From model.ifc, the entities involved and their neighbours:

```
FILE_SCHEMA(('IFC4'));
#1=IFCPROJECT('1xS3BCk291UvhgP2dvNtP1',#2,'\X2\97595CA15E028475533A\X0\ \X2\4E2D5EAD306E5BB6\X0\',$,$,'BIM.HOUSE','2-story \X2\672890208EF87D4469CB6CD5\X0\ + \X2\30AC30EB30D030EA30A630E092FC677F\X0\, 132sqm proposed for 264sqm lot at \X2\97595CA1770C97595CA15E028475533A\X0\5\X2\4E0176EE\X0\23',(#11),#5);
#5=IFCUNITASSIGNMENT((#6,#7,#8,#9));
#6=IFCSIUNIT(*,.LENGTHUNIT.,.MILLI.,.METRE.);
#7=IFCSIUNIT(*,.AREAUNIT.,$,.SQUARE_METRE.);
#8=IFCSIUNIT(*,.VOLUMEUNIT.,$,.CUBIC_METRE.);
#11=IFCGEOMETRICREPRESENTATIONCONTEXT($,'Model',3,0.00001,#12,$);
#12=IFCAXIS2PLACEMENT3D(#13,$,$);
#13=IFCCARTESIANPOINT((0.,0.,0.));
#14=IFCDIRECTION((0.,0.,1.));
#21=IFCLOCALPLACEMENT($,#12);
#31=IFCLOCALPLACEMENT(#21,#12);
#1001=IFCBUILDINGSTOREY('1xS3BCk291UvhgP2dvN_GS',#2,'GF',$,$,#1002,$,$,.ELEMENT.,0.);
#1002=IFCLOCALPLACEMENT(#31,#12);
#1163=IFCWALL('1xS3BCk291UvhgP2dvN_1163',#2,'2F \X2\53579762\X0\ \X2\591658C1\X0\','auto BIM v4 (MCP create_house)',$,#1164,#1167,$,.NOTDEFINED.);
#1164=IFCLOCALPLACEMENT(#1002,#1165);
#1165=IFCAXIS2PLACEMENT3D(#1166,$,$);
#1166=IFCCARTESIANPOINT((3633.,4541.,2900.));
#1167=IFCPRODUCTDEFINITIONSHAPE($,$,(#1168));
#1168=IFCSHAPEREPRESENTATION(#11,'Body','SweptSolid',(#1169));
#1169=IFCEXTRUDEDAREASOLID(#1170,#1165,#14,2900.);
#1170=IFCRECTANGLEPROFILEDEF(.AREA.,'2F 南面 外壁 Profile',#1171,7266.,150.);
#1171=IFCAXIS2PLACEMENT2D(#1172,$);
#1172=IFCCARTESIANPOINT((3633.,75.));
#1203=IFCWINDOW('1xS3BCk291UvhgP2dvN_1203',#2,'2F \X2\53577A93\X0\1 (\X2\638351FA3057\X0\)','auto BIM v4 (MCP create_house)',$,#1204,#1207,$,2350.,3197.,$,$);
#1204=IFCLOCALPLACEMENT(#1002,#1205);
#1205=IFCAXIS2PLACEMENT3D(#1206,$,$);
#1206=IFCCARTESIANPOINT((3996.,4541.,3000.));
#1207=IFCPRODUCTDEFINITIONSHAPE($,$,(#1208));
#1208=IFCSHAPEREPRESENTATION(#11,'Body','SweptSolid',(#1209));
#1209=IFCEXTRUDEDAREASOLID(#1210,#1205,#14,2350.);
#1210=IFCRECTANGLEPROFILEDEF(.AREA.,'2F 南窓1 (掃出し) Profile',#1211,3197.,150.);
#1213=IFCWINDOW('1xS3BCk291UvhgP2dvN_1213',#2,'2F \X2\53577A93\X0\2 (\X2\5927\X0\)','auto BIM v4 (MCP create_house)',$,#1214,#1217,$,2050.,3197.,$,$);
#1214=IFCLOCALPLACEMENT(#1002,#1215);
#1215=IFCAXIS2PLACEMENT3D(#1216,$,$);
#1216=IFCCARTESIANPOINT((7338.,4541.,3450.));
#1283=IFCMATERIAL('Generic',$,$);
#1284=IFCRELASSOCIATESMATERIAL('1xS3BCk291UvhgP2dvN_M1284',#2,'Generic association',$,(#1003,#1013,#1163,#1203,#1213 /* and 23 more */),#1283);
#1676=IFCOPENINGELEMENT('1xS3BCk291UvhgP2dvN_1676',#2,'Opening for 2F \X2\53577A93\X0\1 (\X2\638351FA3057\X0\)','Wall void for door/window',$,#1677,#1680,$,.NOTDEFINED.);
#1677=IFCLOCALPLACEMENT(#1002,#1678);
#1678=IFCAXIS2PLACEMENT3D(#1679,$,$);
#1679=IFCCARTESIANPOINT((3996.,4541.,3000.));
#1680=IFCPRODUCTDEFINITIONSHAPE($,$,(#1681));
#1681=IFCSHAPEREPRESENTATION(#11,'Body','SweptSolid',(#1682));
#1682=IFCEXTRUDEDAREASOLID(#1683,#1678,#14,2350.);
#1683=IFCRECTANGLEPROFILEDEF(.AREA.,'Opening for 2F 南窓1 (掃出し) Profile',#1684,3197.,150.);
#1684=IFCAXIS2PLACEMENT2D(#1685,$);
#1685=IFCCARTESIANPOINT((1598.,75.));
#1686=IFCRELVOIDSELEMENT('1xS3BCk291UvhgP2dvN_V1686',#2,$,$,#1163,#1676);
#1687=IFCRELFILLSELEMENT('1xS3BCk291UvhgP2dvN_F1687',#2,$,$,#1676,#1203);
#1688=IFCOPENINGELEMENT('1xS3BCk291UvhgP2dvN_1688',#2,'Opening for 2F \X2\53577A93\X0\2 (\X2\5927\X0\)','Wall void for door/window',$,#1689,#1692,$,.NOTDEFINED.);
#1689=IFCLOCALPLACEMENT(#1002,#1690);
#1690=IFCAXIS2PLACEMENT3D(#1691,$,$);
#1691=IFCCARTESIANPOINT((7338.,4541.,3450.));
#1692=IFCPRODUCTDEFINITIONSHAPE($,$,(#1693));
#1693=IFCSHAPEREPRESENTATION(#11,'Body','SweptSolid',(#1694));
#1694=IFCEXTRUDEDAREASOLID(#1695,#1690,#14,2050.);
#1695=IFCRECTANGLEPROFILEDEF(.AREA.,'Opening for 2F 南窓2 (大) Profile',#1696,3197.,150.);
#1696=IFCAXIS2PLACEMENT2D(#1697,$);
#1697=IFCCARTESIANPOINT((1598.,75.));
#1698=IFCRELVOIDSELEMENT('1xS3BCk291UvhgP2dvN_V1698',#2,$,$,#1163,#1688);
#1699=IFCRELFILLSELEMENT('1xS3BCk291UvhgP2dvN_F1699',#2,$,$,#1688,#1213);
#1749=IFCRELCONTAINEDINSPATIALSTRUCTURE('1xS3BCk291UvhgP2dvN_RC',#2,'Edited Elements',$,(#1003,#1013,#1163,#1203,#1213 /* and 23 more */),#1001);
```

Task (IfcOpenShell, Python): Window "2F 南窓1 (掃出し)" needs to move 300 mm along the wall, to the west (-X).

```python
import ifcopenshell
import ifcopenshell.api.geometry
import ifcopenshell.util.placement

model = ifcopenshell.open("model.ifc")

window = model.by_guid("1xS3BCk291UvhgP2dvN_1203")
opening = window.FillsVoids[0].RelatingOpeningElement
wall = opening.VoidsElements[0].RelatingBuildingElement

wall_matrix = ifcopenshell.util.placement.get_local_placement(wall.ObjectPlacement)
shift = wall_matrix[:3, 0] * -300.0
before = ifcopenshell.util.placement.get_local_placement(window.ObjectPlacement)[:3, 3].copy()

# The window is not placed relative to its opening, so move both.
for product in (opening, window):
    matrix = ifcopenshell.util.placement.get_local_placement(product.ObjectPlacement)
    matrix[:3, 3] += shift
    ifcopenshell.api.geometry.edit_object_placement(model, product=product, matrix=matrix, is_si=False)

after = ifcopenshell.util.placement.get_local_placement(window.ObjectPlacement)[:3, 3]
print("window moved by", (after - before).round(3) + 0.0)

model.write("model-out.ifc")
```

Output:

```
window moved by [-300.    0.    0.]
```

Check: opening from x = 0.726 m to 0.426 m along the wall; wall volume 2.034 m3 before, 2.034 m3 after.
